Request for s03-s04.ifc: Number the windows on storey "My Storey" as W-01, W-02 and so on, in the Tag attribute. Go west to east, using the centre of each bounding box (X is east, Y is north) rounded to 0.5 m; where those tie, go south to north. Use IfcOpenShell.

First a look at what the model holds.

```python
import ifcopenshell
import ifcopenshell.util.element
import ifcopenshell.util.placement

model = ifcopenshell.open("s03-s04.ifc")
print(model.schema)
storey = next(s for s in model.by_type("IfcBuildingStorey") if s.Name == "My Storey")
windows = [e for e in ifcopenshell.util.element.get_decomposition(storey) if e.is_a("IfcWindow")]
for e in sorted(windows, key=lambda e: e.id()):
    origin = ifcopenshell.util.placement.get_local_placement(e.ObjectPlacement)[:3, 3]
    print(e.id(), e.Tag, e.Name, origin.round(2) + 0.0, sep=" | ")
```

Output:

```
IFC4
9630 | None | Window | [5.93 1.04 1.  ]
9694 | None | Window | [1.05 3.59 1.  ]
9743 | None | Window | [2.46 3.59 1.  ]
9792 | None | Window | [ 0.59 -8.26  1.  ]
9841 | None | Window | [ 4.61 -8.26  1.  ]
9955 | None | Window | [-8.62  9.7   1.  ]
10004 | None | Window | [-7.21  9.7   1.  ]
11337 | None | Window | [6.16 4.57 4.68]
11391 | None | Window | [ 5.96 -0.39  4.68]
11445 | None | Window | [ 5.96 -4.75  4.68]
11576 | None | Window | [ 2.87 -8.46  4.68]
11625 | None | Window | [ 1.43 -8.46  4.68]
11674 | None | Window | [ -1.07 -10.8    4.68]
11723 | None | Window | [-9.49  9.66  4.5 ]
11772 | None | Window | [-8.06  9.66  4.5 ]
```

```python
import ifcopenshell
import ifcopenshell.geom
import ifcopenshell.util.element
import ifcopenshell.util.shape

model = ifcopenshell.open("s03-s04.ifc")
settings = ifcopenshell.geom.settings()
settings.set("use-world-coords", True)


def centre(element):
    shape = ifcopenshell.geom.create_shape(settings, element)
    return ifcopenshell.util.shape.get_bbox_centroid(shape.geometry)


storey = next(s for s in model.by_type("IfcBuildingStorey") if s.Name == "My Storey")
windows = [e for e in ifcopenshell.util.element.get_decomposition(storey) if e.is_a("IfcWindow")]

# Insertion points can sit at a corner or the storey origin, so sort by the geometry (in metres).
centres = {e: centre(e) for e in windows}
windows.sort(key=lambda e: (round(centres[e][0] / 0.5), centres[e][1]))

for i, e in enumerate(windows, start=1):
    number = f"W-{i:02d}"
    e.Tag = number
    print(e.id(), number)

model.write("s03-s04_edited.ifc")
```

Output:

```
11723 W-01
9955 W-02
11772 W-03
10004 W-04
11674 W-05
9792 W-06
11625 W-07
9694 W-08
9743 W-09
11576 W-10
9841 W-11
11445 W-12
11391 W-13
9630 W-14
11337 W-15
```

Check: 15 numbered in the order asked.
